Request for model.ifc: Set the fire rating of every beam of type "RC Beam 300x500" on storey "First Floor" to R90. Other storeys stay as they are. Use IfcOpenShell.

First a look at what the model holds.

```python
import ifcopenshell
import ifcopenshell.util.element

model = ifcopenshell.open("model.ifc")
print(model.schema)
storey = next(s for s in model.by_type("IfcBuildingStorey") if s.Name == "First Floor")
beams = [e for e in ifcopenshell.util.element.get_decomposition(storey) if e.is_a("IfcBeam")]
seen = {}
for e in beams:
    element_type = ifcopenshell.util.element.get_type(e)
    key = (element_type.Name if element_type != e and element_type else None, ifcopenshell.util.element.get_pset(e, "Pset_BeamCommon", "FireRating"))
    seen[key] = seen.get(key, 0) + 1
for (name, value), count in sorted(seen.items(), key=str):
    print(count, "x", name, "|", value)
```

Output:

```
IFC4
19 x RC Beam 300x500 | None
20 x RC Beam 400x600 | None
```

```python
import ifcopenshell
import ifcopenshell.api.pset
import ifcopenshell.util.element

model = ifcopenshell.open("model.ifc")

storey = next(s for s in model.by_type("IfcBuildingStorey") if s.Name == "First Floor")
beams = [e for e in ifcopenshell.util.element.get_decomposition(storey) if e.is_a("IfcBeam")]

count = 0
for e in beams:
    element_type = ifcopenshell.util.element.get_type(e)
    if element_type in (None, e) or element_type.Name != "RC Beam 300x500":
        continue
    # add_pset returns the element's existing set when there is one.
    pset = ifcopenshell.api.pset.add_pset(model, product=e, name="Pset_BeamCommon")
    ifcopenshell.api.pset.edit_pset(model, pset=pset, properties={"FireRating": "R90"})
    count += 1

print(count, "beams updated")

model.write("model_rev.ifc")
```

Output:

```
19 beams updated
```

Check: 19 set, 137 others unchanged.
